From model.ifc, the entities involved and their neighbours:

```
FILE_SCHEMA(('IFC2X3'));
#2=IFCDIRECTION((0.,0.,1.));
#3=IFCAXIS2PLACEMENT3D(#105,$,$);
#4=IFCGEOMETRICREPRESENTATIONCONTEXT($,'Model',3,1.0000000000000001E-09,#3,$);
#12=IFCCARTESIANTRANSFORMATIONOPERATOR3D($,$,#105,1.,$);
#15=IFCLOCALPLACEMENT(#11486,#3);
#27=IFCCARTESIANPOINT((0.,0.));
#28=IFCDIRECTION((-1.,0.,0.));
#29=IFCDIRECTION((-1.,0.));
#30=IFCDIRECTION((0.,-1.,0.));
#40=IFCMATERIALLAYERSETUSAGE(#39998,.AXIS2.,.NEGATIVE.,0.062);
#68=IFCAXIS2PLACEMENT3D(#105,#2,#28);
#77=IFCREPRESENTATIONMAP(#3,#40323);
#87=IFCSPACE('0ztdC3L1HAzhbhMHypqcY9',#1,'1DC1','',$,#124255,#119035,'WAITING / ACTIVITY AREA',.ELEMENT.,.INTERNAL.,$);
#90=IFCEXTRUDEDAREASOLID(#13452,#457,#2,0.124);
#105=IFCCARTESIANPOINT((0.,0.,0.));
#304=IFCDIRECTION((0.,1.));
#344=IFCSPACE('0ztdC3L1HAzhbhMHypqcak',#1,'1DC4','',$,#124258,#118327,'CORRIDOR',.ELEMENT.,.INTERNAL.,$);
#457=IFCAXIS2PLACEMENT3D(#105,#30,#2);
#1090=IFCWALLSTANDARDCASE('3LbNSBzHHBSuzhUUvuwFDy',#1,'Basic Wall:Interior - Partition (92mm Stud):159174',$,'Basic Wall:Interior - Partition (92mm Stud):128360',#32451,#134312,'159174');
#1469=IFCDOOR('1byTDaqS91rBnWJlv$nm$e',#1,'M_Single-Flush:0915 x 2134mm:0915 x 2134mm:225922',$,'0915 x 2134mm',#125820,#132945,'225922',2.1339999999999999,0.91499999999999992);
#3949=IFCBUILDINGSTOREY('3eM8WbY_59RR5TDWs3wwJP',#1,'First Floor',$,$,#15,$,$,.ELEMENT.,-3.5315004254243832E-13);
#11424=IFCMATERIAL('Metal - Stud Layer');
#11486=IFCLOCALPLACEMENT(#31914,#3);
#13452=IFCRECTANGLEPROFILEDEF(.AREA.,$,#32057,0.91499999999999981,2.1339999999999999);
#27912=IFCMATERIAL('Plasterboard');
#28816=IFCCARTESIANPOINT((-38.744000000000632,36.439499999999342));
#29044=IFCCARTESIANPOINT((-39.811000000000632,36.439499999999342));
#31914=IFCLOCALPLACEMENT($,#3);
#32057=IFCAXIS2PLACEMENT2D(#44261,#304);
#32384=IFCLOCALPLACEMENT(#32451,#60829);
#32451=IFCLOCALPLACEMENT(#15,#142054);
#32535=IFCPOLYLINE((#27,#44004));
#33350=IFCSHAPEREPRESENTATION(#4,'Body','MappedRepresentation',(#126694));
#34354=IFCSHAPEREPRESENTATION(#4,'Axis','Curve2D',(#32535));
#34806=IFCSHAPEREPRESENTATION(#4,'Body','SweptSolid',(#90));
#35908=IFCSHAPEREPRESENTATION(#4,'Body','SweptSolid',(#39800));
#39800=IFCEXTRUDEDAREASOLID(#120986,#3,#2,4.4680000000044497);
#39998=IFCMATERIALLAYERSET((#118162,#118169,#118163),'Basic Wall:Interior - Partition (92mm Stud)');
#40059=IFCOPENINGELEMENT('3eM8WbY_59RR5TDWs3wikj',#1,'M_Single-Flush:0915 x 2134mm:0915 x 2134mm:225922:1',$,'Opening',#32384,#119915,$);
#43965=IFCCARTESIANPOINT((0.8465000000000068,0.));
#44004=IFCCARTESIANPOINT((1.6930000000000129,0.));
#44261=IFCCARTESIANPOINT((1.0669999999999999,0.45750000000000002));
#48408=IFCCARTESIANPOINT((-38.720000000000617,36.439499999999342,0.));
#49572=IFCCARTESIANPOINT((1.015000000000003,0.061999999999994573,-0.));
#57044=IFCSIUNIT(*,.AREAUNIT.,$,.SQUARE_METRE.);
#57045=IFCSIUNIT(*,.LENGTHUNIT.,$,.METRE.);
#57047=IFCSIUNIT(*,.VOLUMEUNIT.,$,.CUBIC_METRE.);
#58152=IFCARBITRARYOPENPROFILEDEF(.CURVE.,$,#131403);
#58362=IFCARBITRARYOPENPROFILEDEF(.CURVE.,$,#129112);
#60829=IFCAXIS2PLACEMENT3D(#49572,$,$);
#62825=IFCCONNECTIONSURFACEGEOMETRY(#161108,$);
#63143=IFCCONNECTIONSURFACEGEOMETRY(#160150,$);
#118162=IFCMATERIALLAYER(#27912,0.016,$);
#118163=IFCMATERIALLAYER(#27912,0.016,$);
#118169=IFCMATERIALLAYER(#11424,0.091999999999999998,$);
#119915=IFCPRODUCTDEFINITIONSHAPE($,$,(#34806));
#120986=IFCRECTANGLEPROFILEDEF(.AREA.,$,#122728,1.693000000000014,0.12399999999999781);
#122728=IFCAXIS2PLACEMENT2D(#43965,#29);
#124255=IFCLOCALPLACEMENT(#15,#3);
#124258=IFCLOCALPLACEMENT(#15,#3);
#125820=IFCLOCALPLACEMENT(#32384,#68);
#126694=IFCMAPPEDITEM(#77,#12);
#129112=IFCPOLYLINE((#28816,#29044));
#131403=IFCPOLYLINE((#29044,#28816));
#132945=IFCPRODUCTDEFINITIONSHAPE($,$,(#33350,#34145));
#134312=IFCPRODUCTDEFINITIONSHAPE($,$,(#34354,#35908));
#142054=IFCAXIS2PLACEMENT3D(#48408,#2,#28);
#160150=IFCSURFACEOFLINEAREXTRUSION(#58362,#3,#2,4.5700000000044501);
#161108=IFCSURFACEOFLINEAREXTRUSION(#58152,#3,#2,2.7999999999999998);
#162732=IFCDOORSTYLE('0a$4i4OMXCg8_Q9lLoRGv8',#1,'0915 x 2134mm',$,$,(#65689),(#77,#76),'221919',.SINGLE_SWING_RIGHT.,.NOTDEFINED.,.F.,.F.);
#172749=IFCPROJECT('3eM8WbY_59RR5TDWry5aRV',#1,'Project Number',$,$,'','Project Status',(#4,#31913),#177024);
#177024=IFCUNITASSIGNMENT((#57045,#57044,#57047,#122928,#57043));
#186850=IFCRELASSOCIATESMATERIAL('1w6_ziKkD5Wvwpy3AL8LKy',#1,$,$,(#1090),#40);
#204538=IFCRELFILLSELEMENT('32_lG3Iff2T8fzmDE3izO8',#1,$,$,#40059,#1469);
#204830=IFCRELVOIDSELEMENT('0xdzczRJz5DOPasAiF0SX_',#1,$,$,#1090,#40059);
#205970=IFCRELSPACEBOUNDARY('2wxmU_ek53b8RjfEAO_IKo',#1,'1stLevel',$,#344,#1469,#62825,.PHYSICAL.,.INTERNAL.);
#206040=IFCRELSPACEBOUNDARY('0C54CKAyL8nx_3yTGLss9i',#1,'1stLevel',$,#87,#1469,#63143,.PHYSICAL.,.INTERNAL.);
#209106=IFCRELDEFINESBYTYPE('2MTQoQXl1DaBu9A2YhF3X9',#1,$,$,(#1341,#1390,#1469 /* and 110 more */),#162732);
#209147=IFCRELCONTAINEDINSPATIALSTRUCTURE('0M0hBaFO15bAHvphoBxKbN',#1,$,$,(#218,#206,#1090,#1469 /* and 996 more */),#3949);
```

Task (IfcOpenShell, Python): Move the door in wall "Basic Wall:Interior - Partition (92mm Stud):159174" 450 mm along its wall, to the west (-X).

```python
import numpy as np
import ifcopenshell
import ifcopenshell.api.geometry
import ifcopenshell.util.placement

model = ifcopenshell.open("model.ifc")

door = model.by_id(1469)
opening = door.FillsVoids[0].RelatingOpeningElement
wall = opening.VoidsElements[0].RelatingBuildingElement

wall_matrix = ifcopenshell.util.placement.get_local_placement(wall.ObjectPlacement)
shift = wall_matrix[:3, 0] * 0.45
before = ifcopenshell.util.placement.get_local_placement(door.ObjectPlacement)[:3, 3].copy()

# The door is placed relative to its opening, so it follows when the opening moves.
matrix = ifcopenshell.util.placement.get_local_placement(opening.ObjectPlacement)
matrix[:3, 3] += shift
ifcopenshell.api.geometry.edit_object_placement(
    model, product=opening, matrix=matrix, is_si=False, should_transform_children=True
)

# Space boundary surfaces are stored in each space's coordinates; move them too.
for rel in door.ProvidesBoundaries:
    if not rel.ConnectionGeometry:
        continue
    surface = rel.ConnectionGeometry.SurfaceOnRelatingElement
    space_matrix = ifcopenshell.util.placement.get_local_placement(rel.RelatingSpace.ObjectPlacement)
    point = np.array(surface.Position.Location.Coordinates) + space_matrix[:3, :3].T @ shift
    surface.Position = model.createIfcAxis2Placement3D(
        model.createIfcCartesianPoint(point.tolist()), surface.Position.Axis, surface.Position.RefDirection
    )

after = ifcopenshell.util.placement.get_local_placement(door.ObjectPlacement)[:3, 3]
print("door moved by", (after - before).round(3) + 0.0)

model.write("model-out.ifc")
```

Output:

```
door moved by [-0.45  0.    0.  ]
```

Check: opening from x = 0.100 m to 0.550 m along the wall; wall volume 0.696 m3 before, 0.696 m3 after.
